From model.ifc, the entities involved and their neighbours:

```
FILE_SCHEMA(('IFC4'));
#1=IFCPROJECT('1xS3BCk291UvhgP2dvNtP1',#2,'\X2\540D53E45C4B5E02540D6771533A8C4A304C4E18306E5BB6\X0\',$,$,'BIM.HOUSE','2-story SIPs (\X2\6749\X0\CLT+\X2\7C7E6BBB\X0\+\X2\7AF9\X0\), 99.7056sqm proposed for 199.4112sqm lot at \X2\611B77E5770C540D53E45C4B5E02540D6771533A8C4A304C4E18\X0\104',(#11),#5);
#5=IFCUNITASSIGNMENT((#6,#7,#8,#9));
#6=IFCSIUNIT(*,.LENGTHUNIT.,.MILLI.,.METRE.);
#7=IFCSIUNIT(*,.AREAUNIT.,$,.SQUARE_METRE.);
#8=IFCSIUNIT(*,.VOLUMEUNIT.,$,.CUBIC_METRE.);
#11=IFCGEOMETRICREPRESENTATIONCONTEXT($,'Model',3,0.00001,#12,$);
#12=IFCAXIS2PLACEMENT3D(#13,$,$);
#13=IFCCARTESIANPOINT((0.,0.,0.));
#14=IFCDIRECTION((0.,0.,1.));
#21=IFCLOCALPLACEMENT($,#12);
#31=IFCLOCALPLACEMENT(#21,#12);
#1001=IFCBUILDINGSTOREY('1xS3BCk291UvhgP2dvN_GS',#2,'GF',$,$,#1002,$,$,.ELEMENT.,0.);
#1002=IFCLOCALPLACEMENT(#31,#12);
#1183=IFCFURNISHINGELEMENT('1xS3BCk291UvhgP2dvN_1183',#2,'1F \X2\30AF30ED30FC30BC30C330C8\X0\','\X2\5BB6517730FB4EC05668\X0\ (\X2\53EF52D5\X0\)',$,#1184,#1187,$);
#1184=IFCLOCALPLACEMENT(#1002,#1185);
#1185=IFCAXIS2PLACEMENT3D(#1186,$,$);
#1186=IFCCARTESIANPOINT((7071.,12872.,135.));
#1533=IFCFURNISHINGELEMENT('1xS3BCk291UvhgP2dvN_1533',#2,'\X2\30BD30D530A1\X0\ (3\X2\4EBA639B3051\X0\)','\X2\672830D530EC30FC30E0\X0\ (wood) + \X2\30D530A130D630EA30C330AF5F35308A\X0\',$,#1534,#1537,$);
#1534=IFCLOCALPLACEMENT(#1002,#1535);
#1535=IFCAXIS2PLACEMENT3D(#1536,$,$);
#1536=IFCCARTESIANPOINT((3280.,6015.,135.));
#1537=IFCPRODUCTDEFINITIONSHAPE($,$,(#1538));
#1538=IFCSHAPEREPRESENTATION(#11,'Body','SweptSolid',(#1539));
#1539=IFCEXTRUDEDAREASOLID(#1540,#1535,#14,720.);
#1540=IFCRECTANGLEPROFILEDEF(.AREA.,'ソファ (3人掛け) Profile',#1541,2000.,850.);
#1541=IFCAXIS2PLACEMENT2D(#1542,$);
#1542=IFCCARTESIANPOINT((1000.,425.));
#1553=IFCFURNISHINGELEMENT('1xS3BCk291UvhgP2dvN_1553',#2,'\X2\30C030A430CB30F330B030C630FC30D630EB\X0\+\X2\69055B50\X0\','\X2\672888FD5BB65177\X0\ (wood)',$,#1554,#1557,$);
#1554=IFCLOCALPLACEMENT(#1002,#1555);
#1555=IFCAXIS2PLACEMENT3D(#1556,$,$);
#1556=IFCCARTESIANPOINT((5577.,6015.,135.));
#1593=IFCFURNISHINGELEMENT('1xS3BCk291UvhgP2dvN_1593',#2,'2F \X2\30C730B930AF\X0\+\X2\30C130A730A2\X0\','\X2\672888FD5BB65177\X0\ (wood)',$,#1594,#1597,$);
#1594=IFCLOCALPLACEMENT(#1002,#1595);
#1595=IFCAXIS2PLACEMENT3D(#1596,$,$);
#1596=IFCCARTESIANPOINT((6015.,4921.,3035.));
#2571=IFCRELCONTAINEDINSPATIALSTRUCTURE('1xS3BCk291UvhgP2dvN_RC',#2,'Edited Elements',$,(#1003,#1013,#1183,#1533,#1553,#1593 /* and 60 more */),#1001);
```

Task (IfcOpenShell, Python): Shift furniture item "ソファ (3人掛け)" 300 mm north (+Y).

```python
import ifcopenshell
import ifcopenshell.api.geometry
import ifcopenshell.util.placement

model = ifcopenshell.open("model.ifc")

item = model.by_guid("1xS3BCk291UvhgP2dvN_1533")
matrix = ifcopenshell.util.placement.get_local_placement(item.ObjectPlacement)
matrix[1, 3] += 300.0
ifcopenshell.api.geometry.edit_object_placement(model, product=item, matrix=matrix, is_si=False)

print(ifcopenshell.util.placement.get_local_placement(item.ObjectPlacement).round(3) + 0.0)

model.write("model_v2.ifc")
```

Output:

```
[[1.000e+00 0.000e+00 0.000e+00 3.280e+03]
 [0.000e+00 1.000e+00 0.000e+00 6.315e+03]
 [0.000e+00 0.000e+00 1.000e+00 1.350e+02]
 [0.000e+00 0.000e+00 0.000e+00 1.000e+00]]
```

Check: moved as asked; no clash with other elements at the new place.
